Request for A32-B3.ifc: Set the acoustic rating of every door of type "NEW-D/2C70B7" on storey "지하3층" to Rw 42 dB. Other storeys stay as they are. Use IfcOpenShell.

First a look at what the model holds.

```python
import ifcopenshell
import ifcopenshell.util.element

model = ifcopenshell.open("A32-B3.ifc")
print(model.schema)
storey = next(s for s in model.by_type("IfcBuildingStorey") if s.Name == "지하3층")
doors = [e for e in ifcopenshell.util.element.get_decomposition(storey) if e.is_a("IfcDoor")]
seen = {}
for e in doors:
    element_type = ifcopenshell.util.element.get_type(e)
    key = (element_type.Name if element_type != e and element_type else None, ifcopenshell.util.element.get_pset(e, "Pset_DoorCommon", "AcousticRating"))
    seen[key] = seen.get(key, 0) + 1
for (name, value), count in sorted(seen.items(), key=str):
    print(count, "x", name, "|", value)
```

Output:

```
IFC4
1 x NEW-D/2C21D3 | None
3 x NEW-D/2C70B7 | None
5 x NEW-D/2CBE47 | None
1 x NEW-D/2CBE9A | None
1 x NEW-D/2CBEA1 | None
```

```python
import ifcopenshell
import ifcopenshell.api.pset
import ifcopenshell.util.element

model = ifcopenshell.open("A32-B3.ifc")

storey = next(s for s in model.by_type("IfcBuildingStorey") if s.Name == "지하3층")
doors = [e for e in ifcopenshell.util.element.get_decomposition(storey) if e.is_a("IfcDoor")]

count = 0
for e in doors:
    element_type = ifcopenshell.util.element.get_type(e)
    if element_type in (None, e) or element_type.Name != "NEW-D/2C70B7":
        continue
    # add_pset returns the element's existing set when there is one.
    pset = ifcopenshell.api.pset.add_pset(model, product=e, name="Pset_DoorCommon")
    ifcopenshell.api.pset.edit_pset(model, pset=pset, properties={"AcousticRating": "Rw 42 dB"})
    count += 1

print(count, "doors updated")

model.write("A32-B3_rev.ifc")
```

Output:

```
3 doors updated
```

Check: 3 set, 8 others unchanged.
